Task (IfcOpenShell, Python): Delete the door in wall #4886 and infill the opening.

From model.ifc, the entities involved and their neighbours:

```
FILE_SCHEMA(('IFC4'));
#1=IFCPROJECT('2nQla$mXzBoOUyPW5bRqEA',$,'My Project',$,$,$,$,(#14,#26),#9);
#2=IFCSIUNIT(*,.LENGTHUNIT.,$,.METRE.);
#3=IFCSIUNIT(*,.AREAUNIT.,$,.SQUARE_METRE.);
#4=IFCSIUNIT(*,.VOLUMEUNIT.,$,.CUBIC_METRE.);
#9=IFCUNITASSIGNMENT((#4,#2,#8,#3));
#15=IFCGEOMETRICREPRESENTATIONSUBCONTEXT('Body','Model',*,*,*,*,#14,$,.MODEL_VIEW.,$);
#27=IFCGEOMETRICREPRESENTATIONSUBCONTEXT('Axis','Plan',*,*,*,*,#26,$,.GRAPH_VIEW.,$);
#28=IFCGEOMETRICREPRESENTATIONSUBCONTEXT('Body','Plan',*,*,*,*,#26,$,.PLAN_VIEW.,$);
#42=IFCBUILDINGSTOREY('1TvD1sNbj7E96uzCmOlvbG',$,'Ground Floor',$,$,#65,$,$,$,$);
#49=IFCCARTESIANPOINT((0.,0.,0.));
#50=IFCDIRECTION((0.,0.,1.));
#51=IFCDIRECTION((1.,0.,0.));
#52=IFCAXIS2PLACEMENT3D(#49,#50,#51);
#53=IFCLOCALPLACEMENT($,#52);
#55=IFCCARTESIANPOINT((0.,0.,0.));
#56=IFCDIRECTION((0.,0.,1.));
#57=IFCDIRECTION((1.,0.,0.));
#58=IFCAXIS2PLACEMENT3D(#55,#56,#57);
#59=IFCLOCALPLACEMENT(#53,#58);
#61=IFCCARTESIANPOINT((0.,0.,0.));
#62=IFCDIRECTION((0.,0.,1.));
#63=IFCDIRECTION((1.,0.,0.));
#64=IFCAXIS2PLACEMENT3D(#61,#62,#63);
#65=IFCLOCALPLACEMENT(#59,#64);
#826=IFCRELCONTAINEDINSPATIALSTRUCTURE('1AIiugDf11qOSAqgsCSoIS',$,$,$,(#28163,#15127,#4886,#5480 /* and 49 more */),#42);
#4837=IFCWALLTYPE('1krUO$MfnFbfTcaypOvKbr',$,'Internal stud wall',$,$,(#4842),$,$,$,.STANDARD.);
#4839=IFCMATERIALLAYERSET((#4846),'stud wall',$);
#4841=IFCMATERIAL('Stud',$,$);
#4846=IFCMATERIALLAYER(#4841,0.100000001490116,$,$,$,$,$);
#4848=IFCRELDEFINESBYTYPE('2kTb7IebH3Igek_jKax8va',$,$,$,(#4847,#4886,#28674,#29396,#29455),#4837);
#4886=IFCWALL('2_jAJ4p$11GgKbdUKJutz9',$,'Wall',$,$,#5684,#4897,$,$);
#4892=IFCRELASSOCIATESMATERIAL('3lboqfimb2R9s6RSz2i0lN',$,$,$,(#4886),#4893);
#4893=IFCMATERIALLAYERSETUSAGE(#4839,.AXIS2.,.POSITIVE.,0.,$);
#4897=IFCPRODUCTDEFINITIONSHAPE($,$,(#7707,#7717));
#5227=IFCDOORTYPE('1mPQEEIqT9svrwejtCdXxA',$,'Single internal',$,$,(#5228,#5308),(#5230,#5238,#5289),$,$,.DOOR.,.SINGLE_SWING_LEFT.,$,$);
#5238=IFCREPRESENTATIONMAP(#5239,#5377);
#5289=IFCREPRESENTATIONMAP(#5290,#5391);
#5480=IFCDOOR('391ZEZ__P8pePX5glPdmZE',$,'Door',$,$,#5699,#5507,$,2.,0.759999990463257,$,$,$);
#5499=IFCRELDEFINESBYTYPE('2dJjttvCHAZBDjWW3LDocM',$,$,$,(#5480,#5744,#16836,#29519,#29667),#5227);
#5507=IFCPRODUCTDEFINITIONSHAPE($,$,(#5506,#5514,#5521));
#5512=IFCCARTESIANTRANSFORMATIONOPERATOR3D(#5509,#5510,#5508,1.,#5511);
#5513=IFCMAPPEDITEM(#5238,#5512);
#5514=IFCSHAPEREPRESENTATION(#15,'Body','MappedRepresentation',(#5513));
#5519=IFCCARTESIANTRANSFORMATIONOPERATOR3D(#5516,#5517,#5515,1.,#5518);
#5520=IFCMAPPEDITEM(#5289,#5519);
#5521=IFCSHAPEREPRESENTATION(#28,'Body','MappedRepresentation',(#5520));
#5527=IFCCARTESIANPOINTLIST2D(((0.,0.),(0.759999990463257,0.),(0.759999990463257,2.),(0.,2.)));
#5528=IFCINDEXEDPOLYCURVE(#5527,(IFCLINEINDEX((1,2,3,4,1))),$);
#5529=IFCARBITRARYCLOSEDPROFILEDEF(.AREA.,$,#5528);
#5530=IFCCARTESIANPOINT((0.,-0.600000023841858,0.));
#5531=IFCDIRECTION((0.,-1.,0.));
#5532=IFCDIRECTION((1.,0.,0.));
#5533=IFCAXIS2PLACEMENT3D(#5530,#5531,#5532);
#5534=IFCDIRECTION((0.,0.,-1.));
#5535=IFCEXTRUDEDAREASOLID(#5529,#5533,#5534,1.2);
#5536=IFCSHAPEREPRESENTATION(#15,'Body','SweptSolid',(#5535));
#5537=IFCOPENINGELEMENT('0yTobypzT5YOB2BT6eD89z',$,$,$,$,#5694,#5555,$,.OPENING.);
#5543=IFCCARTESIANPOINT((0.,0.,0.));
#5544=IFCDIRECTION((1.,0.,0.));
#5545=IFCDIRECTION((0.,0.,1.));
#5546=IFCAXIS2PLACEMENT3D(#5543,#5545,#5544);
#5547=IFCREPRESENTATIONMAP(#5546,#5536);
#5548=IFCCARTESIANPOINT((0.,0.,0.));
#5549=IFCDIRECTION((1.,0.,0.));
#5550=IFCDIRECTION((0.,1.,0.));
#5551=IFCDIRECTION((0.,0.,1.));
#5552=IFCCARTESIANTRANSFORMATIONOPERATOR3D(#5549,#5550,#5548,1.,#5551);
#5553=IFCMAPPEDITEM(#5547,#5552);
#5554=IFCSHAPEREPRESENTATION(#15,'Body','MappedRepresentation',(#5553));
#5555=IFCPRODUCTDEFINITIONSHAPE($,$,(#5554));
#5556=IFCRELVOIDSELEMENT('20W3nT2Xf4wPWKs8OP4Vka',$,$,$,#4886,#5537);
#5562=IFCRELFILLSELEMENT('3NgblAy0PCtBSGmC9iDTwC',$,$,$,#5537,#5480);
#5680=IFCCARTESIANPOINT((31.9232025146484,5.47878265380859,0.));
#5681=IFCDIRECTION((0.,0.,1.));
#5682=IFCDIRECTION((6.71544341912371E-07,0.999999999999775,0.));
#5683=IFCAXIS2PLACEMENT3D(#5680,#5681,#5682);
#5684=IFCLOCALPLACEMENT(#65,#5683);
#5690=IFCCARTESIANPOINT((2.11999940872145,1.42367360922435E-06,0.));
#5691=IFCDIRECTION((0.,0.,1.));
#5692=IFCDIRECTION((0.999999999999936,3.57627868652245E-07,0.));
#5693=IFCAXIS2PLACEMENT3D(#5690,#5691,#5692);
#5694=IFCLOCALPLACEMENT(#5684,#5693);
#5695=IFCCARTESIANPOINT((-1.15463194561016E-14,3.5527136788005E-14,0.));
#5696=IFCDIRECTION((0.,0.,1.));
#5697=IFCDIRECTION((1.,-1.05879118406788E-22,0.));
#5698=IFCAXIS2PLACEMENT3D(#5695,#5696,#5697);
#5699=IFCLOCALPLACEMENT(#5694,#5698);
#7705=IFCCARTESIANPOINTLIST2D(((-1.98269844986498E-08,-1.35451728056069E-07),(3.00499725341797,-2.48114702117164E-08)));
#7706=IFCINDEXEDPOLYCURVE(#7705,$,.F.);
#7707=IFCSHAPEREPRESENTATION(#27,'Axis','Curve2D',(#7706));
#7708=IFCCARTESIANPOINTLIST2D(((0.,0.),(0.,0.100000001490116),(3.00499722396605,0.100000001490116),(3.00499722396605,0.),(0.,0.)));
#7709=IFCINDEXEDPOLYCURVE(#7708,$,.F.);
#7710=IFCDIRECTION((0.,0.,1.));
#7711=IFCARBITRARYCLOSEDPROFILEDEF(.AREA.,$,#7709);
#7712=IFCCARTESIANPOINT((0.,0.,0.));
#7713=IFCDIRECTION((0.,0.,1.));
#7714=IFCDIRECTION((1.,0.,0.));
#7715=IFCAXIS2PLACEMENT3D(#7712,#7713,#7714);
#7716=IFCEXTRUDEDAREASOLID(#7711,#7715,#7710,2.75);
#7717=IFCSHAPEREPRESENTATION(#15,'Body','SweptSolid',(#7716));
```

```python
import ifcopenshell
import ifcopenshell.api.feature
import ifcopenshell.api.root
import ifcopenshell.geom
import ifcopenshell.util.shape

model = ifcopenshell.open("model.ifc")
settings = ifcopenshell.geom.settings()


def volume(element):
    """Net volume in cubic metres, openings subtracted."""
    shape = ifcopenshell.geom.create_shape(settings, element)
    return ifcopenshell.util.shape.get_volume(shape.geometry)


door = model.by_guid("391ZEZ__P8pePX5glPdmZE")
opening = door.FillsVoids[0].RelatingOpeningElement
wall = opening.VoidsElements[0].RelatingBuildingElement
before = volume(wall)

ifcopenshell.api.root.remove_product(model, product=door)
ifcopenshell.api.feature.remove_feature(model, feature=opening)

after = volume(wall)

print(f"wall volume {before:.3f} -> {after:.3f} m3")

model.write("model-out.ifc")
```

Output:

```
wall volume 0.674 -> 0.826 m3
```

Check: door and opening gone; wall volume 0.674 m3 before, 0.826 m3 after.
